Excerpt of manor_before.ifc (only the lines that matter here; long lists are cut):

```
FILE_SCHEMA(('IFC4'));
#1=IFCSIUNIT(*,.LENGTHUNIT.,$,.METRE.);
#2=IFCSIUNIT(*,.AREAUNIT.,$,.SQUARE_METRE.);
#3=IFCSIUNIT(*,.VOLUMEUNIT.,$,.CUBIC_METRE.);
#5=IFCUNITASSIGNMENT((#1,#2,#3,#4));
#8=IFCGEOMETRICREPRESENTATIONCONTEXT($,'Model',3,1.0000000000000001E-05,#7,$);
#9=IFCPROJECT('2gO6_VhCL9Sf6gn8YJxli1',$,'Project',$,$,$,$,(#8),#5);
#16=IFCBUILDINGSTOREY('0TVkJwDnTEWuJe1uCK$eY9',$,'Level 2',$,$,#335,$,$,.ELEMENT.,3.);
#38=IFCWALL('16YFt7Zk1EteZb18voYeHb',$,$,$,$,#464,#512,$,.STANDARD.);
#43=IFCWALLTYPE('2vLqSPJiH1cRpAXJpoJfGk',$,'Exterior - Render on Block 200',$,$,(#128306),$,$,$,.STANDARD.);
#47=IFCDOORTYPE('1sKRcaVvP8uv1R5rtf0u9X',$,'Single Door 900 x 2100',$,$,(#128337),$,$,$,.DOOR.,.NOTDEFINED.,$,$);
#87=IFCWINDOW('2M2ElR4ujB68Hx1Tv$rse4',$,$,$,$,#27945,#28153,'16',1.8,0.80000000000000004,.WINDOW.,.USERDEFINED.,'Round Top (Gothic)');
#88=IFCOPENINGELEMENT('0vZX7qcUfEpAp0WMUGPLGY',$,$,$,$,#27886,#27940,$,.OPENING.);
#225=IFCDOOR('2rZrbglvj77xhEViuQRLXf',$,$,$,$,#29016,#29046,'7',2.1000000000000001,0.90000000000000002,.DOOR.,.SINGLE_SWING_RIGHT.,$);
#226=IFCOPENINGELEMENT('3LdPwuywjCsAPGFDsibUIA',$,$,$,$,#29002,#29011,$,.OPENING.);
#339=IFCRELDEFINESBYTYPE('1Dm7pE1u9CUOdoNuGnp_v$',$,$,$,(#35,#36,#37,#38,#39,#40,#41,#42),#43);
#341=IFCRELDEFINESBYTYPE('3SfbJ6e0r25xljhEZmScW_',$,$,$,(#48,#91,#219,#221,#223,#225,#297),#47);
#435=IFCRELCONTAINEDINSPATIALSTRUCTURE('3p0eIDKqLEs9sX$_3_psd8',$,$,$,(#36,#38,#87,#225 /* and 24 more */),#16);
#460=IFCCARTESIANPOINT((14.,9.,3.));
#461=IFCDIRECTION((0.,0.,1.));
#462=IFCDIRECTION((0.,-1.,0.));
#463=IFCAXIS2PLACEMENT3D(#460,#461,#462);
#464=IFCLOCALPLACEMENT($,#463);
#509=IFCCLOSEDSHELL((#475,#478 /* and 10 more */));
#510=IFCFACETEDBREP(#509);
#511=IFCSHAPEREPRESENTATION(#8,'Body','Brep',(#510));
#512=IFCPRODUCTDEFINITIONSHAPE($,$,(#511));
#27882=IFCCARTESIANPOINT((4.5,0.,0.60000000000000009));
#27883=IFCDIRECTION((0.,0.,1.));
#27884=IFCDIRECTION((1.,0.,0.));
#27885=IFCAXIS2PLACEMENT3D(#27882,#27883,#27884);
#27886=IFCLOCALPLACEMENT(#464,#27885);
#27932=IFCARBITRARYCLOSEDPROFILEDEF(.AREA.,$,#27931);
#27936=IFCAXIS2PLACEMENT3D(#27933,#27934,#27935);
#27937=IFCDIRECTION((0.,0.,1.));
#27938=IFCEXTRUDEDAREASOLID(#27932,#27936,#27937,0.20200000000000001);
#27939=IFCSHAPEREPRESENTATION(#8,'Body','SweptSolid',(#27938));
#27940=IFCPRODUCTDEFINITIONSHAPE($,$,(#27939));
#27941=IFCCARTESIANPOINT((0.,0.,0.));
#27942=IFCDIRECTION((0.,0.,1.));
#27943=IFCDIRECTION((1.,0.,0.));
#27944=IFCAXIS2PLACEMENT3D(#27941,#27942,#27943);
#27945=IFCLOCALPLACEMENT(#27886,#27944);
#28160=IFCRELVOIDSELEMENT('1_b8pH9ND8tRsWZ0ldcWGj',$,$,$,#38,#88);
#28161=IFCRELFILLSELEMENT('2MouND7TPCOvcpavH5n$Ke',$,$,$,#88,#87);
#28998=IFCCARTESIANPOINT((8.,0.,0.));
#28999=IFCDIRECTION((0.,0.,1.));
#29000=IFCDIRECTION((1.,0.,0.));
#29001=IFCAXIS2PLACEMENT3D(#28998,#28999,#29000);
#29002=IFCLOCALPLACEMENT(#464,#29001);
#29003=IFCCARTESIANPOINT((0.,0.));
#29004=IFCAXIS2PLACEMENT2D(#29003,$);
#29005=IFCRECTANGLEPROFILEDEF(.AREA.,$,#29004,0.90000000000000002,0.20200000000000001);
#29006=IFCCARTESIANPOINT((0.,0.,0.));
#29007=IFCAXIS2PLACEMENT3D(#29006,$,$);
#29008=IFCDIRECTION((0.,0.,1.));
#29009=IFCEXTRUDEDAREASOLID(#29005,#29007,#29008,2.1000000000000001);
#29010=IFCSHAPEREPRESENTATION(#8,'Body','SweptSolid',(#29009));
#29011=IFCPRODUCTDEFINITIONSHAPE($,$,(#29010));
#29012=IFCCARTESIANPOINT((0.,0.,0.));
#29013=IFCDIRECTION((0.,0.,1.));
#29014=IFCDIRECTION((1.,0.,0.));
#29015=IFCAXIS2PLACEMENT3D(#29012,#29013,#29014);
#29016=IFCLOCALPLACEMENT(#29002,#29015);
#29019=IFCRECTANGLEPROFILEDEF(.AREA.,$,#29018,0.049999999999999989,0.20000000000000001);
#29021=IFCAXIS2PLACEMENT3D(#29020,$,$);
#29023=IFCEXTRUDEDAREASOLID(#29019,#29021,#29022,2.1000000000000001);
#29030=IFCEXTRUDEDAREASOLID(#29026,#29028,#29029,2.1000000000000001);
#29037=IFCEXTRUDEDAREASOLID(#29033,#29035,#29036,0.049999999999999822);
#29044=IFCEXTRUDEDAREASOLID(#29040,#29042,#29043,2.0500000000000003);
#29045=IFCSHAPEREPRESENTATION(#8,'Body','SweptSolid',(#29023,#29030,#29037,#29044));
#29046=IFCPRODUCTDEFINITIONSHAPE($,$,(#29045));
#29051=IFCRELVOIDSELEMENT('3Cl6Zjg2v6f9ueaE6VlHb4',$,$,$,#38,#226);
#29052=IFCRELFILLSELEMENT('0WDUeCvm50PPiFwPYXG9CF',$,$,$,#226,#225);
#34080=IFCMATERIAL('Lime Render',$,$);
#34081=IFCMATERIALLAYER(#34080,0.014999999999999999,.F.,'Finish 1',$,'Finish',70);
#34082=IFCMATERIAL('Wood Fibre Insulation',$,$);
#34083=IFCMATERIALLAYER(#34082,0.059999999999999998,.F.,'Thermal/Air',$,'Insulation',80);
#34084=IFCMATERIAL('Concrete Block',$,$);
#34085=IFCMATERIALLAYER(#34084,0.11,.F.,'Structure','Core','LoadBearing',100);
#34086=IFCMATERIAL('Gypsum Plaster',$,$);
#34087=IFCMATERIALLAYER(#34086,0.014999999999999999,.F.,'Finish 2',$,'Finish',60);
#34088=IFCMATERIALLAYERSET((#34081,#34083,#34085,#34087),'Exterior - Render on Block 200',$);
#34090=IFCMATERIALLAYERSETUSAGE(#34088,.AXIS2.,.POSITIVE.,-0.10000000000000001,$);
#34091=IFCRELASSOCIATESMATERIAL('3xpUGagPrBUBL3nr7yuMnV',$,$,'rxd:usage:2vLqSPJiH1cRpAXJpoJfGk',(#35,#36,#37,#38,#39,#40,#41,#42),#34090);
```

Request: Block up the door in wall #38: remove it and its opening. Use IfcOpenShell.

```python
import ifcopenshell
import ifcopenshell.api.feature
import ifcopenshell.api.root
import ifcopenshell.geom
import ifcopenshell.util.shape

model = ifcopenshell.open("manor_before.ifc")
settings = ifcopenshell.geom.settings()


def volume(element):
    """Net volume in cubic metres, openings subtracted."""
    shape = ifcopenshell.geom.create_shape(settings, element)
    return ifcopenshell.util.shape.get_volume(shape.geometry)


door = model.by_id(225)
opening = door.FillsVoids[0].RelatingOpeningElement
wall = opening.VoidsElements[0].RelatingBuildingElement
before = volume(wall)

ifcopenshell.api.root.remove_product(model, product=door)
ifcopenshell.api.feature.remove_feature(model, feature=opening)

after = volume(wall)

print(f"wall volume {before:.3f} -> {after:.3f} m3")

model.write("manor_before_rev.ifc")
```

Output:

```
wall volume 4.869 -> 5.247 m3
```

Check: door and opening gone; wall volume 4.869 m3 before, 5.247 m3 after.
